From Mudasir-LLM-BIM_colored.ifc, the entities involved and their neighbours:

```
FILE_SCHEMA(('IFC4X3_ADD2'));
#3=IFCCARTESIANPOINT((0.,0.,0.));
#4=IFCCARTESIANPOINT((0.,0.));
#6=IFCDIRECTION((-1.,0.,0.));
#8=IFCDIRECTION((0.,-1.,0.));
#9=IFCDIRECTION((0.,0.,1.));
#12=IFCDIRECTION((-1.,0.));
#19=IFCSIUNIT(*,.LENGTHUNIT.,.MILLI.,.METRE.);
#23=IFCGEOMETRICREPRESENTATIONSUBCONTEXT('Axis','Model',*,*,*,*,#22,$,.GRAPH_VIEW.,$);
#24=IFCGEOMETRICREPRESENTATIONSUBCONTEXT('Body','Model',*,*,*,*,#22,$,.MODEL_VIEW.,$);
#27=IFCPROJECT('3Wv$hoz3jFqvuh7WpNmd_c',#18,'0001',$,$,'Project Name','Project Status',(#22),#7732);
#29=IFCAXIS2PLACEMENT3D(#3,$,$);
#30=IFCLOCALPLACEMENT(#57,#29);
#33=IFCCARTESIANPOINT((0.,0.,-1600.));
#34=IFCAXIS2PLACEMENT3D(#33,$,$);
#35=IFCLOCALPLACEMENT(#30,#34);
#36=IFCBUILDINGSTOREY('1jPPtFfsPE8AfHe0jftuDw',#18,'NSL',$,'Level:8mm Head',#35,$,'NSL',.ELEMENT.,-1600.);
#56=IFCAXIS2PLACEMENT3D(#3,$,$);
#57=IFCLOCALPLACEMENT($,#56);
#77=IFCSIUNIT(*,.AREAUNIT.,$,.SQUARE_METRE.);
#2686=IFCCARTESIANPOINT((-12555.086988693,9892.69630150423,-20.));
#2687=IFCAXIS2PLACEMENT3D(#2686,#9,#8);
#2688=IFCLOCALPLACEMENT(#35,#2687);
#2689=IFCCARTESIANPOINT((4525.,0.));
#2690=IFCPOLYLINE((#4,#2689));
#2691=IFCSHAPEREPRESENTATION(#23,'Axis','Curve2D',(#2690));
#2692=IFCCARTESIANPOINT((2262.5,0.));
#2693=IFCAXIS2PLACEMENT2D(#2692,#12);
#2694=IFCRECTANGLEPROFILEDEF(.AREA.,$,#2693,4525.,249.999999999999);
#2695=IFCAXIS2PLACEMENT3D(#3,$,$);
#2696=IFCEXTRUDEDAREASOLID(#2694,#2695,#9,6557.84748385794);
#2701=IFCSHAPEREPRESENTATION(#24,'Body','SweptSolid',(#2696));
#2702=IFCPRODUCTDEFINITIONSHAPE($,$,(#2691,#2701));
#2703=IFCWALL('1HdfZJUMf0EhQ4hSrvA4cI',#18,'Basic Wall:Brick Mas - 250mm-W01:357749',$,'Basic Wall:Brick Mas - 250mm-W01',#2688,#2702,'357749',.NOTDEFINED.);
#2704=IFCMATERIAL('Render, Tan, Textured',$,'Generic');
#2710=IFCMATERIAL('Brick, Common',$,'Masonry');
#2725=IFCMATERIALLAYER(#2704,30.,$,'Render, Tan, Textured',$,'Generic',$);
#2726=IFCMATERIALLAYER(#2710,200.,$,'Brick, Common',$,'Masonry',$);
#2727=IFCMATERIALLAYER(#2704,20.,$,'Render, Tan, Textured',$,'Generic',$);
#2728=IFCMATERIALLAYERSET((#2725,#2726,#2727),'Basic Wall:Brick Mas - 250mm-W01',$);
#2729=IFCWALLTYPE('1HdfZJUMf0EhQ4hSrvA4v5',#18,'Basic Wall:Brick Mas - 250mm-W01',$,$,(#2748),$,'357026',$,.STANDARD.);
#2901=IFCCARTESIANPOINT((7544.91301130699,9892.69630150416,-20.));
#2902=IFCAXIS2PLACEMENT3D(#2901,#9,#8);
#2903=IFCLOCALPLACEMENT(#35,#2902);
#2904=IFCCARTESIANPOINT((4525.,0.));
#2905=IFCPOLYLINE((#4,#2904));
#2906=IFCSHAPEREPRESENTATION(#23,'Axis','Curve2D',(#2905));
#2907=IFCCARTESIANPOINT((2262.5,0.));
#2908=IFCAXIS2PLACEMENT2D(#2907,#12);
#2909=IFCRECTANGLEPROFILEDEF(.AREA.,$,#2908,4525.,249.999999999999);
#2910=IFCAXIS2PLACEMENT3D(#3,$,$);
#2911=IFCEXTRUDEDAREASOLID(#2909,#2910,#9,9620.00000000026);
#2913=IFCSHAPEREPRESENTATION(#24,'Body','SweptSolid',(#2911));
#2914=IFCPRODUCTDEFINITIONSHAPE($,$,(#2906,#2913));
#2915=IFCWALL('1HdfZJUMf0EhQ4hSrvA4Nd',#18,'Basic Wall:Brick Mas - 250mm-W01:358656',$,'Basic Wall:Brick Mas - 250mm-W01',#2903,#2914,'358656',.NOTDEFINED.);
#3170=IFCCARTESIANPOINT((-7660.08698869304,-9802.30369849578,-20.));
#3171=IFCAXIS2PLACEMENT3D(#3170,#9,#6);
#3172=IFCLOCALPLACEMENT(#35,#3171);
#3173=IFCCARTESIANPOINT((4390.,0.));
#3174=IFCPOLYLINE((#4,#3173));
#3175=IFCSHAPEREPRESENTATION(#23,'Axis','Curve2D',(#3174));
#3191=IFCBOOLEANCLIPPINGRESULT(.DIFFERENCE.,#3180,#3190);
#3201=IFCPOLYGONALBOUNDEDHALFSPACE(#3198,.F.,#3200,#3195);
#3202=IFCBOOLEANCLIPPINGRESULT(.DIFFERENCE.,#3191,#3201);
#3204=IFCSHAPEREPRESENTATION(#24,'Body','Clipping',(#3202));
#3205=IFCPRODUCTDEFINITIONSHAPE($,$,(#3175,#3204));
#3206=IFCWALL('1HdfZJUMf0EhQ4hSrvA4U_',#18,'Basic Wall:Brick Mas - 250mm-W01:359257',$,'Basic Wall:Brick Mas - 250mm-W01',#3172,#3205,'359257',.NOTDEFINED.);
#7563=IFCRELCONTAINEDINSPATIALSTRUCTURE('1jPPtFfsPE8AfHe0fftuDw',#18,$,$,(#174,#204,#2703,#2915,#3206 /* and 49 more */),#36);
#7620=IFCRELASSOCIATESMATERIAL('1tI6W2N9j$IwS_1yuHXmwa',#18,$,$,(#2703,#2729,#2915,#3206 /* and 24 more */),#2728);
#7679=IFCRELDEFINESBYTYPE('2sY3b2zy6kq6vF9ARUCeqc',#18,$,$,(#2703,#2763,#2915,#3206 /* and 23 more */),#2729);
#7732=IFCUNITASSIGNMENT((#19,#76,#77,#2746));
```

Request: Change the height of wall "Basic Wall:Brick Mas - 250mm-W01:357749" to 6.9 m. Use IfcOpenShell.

```python
import ifcopenshell
import ifcopenshell.geom
import ifcopenshell.util.representation
import ifcopenshell.util.shape
import ifcopenshell.util.unit

model = ifcopenshell.open("Mudasir-LLM-BIM_colored.ifc")
unit_scale = ifcopenshell.util.unit.calculate_unit_scale(model)
settings = ifcopenshell.geom.settings()


def volume(element):
    """Net volume in cubic metres, openings subtracted."""
    shape = ifcopenshell.geom.create_shape(settings, element)
    return ifcopenshell.util.shape.get_volume(shape.geometry)


wall = model.by_guid("1HdfZJUMf0EhQ4hSrvA4cI")
before = volume(wall)

body = ifcopenshell.util.representation.get_representation(wall, "Model", "Body")
solid = body.Items[0]
old_height = solid.Depth
solid.Depth = 6.9 / unit_scale
after = volume(wall)

print(f"height {old_height:g} -> {solid.Depth:g}, volume {before:.3f} -> {after:.3f} m3")

model.write("Mudasir-LLM-BIM_colored_updated.ifc")
```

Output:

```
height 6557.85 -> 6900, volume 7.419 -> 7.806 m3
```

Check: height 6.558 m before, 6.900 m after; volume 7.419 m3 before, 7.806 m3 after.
